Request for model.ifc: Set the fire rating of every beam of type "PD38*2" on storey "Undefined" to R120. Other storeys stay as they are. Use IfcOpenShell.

First a look at what the model holds.

```python
import ifcopenshell
import ifcopenshell.util.element

model = ifcopenshell.open("model.ifc")
print(model.schema)
storey = next(s for s in model.by_type("IfcBuildingStorey") if s.Name == "Undefined")
beams = [e for e in ifcopenshell.util.element.get_decomposition(storey) if e.is_a("IfcBeam")]
seen = {}
for e in beams:
    element_type = ifcopenshell.util.element.get_type(e)
    key = (element_type.Name if element_type != e and element_type else None, ifcopenshell.util.element.get_pset(e, "Pset_BeamCommon", "FireRating"))
    seen[key] = seen.get(key, 0) + 1
for (name, value), count in sorted(seen.items(), key=str):
    print(count, "x", name, "|", value)
```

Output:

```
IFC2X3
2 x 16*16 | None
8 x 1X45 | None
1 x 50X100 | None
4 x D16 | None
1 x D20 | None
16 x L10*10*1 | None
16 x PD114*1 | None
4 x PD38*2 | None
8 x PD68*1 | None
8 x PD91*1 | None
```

```python
import ifcopenshell
import ifcopenshell.api.pset
import ifcopenshell.util.element

model = ifcopenshell.open("model.ifc")

storey = next(s for s in model.by_type("IfcBuildingStorey") if s.Name == "Undefined")
beams = [e for e in ifcopenshell.util.element.get_decomposition(storey) if e.is_a("IfcBeam")]

count = 0
for e in beams:
    element_type = ifcopenshell.util.element.get_type(e)
    if element_type in (None, e) or element_type.Name != "PD38*2":
        continue
    # add_pset returns the element's existing set when there is one.
    pset = ifcopenshell.api.pset.add_pset(model, product=e, name="Pset_BeamCommon")
    ifcopenshell.api.pset.edit_pset(model, pset=pset, properties={"FireRating": "R120"})
    count += 1

print(count, "beams updated")

model.write("model_rev.ifc")
```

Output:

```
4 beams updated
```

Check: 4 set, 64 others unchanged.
